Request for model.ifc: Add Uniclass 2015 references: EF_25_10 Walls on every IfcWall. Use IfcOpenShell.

First a look at what the model holds.

```python
import ifcopenshell

model = ifcopenshell.open("model.ifc")
print(model.schema)
print("classifications:", [c.Name for c in model.by_type("IfcClassification")])
for ifc_class in ("IfcDoor", "IfcRoof", "IfcStair", "IfcWall", "IfcWindow"):
    print(ifc_class, len(model.by_type(ifc_class)))
```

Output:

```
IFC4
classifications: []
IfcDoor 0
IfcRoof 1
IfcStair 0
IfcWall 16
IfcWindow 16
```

```python
import ifcopenshell
import ifcopenshell.api.classification

model = ifcopenshell.open("model.ifc")

system = ifcopenshell.api.classification.add_classification(model, classification="Uniclass 2015")

codes = {
    "IfcWall": ("EF_25_10", "Walls"),
}
for ifc_class, (code, name) in codes.items():
    products = model.by_type(ifc_class)
    ifcopenshell.api.classification.add_reference(
        model, products=products, classification=system, identification=code, name=name
    )
    print(code, len(products))

model.write("model_edited.ifc")
```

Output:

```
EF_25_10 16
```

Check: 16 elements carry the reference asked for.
